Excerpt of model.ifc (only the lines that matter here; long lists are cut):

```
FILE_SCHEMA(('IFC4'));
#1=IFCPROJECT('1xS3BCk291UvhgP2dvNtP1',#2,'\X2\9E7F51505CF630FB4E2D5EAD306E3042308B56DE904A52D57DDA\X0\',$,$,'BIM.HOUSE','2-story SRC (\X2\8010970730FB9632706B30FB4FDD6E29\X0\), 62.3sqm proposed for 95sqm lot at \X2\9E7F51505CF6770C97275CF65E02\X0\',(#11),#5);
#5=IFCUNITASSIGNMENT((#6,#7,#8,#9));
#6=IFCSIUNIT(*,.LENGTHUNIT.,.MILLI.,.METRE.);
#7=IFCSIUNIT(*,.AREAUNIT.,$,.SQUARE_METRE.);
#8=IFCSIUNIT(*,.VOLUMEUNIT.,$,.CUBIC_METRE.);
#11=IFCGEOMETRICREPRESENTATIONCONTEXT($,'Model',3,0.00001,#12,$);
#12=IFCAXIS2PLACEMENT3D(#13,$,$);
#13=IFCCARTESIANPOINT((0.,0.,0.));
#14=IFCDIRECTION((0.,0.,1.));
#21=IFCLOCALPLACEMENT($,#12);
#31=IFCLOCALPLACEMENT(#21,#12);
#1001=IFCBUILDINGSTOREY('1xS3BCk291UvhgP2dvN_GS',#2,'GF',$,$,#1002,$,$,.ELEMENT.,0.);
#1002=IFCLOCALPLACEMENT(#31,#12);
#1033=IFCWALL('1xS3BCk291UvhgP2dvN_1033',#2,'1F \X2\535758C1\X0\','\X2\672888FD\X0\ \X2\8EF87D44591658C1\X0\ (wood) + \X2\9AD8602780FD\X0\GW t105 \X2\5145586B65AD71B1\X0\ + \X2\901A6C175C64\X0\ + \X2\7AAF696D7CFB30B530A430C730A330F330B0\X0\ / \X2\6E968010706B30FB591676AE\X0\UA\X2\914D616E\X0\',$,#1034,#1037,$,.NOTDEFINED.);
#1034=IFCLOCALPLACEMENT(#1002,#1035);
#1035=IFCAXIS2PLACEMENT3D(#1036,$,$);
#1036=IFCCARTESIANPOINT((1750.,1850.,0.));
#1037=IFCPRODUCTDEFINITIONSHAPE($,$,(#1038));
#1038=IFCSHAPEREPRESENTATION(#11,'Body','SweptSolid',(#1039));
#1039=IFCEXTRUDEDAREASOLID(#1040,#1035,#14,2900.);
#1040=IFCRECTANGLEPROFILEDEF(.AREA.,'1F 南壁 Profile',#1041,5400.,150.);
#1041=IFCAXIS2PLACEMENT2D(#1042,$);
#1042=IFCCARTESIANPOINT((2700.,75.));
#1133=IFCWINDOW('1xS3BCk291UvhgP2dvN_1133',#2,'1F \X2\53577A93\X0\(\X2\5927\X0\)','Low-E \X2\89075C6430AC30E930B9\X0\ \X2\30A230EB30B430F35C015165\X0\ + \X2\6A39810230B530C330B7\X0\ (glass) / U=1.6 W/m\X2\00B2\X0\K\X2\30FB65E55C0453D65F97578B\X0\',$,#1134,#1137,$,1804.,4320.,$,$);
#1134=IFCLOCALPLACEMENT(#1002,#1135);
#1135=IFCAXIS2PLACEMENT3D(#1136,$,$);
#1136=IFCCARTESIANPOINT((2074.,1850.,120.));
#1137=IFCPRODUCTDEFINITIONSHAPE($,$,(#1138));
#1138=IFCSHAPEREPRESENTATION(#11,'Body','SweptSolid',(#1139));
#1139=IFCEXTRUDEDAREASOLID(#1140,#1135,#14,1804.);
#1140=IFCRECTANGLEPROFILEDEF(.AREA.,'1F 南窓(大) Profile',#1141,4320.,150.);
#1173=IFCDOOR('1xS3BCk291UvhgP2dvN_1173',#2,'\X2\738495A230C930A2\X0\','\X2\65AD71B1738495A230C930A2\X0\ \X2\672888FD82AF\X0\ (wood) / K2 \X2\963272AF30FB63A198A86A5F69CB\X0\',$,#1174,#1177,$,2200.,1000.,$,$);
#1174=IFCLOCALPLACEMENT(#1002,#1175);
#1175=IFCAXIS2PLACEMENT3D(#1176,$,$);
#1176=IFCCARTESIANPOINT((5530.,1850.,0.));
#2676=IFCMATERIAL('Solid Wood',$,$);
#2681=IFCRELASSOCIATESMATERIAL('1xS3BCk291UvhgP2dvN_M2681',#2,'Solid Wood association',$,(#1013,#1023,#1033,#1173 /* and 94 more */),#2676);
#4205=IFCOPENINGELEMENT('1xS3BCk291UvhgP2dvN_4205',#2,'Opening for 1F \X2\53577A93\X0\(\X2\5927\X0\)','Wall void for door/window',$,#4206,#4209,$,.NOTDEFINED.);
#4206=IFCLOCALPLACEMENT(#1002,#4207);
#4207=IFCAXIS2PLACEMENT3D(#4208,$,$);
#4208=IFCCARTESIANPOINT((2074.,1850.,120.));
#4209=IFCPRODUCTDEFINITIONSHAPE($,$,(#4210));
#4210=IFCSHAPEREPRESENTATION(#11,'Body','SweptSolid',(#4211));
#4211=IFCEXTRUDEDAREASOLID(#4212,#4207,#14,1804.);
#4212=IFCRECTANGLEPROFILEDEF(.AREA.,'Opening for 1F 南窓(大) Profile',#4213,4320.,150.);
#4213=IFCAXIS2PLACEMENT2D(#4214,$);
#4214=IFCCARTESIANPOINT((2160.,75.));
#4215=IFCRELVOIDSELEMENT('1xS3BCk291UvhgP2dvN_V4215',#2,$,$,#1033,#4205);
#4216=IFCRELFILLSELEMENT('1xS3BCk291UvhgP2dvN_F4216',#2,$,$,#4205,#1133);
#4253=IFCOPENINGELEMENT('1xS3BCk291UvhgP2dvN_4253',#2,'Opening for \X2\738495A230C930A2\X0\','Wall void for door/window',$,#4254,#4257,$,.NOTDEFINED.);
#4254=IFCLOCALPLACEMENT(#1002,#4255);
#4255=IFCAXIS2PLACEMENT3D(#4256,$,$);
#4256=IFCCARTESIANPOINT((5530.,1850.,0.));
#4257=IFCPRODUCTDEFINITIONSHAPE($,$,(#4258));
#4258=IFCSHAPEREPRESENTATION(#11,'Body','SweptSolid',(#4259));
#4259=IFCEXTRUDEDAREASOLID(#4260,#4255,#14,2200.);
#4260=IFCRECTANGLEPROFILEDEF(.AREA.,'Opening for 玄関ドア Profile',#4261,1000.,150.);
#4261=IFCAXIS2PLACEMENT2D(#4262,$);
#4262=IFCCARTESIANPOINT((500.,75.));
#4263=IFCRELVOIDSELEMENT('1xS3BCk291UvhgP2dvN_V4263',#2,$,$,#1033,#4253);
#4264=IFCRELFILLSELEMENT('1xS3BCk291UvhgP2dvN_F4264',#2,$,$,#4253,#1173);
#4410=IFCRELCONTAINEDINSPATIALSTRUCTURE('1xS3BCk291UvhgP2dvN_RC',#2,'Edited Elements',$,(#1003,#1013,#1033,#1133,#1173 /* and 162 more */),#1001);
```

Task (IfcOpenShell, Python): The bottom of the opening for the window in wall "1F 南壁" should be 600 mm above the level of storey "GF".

```python
import numpy as np
import ifcopenshell
import ifcopenshell.api.geometry
import ifcopenshell.geom
import ifcopenshell.util.element
import ifcopenshell.util.placement
import ifcopenshell.util.shape
import ifcopenshell.util.unit

model = ifcopenshell.open("model.ifc")
unit_scale = ifcopenshell.util.unit.calculate_unit_scale(model)

window = model.by_id(1133)
opening = window.FillsVoids[0].RelatingOpeningElement
storey = ifcopenshell.util.element.get_container(window, ifc_class="IfcBuildingStorey")
level = ifcopenshell.util.placement.get_local_placement(storey.ObjectPlacement)[2, 3]

# The opening's origin need not be at the sill, so measure its lowest point.
shape = ifcopenshell.geom.create_shape(ifcopenshell.geom.settings(), opening)
bottom = ifcopenshell.util.shape.get_shape_bottom_elevation(shape, shape.geometry) / unit_scale
dz = level + 600.0 - bottom

shift = np.array([0.0, 0.0, dz])
# The window is not placed relative to its opening, so move both.
for product in (opening, window):
    matrix = ifcopenshell.util.placement.get_local_placement(product.ObjectPlacement)
    matrix[:3, 3] += shift
    ifcopenshell.api.geometry.edit_object_placement(model, product=product, matrix=matrix, is_si=False)

print(f"moved by {dz * unit_scale:+.3f} m")

model.write("model_edited.ifc")
```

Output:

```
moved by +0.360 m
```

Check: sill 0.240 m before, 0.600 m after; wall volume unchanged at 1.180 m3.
